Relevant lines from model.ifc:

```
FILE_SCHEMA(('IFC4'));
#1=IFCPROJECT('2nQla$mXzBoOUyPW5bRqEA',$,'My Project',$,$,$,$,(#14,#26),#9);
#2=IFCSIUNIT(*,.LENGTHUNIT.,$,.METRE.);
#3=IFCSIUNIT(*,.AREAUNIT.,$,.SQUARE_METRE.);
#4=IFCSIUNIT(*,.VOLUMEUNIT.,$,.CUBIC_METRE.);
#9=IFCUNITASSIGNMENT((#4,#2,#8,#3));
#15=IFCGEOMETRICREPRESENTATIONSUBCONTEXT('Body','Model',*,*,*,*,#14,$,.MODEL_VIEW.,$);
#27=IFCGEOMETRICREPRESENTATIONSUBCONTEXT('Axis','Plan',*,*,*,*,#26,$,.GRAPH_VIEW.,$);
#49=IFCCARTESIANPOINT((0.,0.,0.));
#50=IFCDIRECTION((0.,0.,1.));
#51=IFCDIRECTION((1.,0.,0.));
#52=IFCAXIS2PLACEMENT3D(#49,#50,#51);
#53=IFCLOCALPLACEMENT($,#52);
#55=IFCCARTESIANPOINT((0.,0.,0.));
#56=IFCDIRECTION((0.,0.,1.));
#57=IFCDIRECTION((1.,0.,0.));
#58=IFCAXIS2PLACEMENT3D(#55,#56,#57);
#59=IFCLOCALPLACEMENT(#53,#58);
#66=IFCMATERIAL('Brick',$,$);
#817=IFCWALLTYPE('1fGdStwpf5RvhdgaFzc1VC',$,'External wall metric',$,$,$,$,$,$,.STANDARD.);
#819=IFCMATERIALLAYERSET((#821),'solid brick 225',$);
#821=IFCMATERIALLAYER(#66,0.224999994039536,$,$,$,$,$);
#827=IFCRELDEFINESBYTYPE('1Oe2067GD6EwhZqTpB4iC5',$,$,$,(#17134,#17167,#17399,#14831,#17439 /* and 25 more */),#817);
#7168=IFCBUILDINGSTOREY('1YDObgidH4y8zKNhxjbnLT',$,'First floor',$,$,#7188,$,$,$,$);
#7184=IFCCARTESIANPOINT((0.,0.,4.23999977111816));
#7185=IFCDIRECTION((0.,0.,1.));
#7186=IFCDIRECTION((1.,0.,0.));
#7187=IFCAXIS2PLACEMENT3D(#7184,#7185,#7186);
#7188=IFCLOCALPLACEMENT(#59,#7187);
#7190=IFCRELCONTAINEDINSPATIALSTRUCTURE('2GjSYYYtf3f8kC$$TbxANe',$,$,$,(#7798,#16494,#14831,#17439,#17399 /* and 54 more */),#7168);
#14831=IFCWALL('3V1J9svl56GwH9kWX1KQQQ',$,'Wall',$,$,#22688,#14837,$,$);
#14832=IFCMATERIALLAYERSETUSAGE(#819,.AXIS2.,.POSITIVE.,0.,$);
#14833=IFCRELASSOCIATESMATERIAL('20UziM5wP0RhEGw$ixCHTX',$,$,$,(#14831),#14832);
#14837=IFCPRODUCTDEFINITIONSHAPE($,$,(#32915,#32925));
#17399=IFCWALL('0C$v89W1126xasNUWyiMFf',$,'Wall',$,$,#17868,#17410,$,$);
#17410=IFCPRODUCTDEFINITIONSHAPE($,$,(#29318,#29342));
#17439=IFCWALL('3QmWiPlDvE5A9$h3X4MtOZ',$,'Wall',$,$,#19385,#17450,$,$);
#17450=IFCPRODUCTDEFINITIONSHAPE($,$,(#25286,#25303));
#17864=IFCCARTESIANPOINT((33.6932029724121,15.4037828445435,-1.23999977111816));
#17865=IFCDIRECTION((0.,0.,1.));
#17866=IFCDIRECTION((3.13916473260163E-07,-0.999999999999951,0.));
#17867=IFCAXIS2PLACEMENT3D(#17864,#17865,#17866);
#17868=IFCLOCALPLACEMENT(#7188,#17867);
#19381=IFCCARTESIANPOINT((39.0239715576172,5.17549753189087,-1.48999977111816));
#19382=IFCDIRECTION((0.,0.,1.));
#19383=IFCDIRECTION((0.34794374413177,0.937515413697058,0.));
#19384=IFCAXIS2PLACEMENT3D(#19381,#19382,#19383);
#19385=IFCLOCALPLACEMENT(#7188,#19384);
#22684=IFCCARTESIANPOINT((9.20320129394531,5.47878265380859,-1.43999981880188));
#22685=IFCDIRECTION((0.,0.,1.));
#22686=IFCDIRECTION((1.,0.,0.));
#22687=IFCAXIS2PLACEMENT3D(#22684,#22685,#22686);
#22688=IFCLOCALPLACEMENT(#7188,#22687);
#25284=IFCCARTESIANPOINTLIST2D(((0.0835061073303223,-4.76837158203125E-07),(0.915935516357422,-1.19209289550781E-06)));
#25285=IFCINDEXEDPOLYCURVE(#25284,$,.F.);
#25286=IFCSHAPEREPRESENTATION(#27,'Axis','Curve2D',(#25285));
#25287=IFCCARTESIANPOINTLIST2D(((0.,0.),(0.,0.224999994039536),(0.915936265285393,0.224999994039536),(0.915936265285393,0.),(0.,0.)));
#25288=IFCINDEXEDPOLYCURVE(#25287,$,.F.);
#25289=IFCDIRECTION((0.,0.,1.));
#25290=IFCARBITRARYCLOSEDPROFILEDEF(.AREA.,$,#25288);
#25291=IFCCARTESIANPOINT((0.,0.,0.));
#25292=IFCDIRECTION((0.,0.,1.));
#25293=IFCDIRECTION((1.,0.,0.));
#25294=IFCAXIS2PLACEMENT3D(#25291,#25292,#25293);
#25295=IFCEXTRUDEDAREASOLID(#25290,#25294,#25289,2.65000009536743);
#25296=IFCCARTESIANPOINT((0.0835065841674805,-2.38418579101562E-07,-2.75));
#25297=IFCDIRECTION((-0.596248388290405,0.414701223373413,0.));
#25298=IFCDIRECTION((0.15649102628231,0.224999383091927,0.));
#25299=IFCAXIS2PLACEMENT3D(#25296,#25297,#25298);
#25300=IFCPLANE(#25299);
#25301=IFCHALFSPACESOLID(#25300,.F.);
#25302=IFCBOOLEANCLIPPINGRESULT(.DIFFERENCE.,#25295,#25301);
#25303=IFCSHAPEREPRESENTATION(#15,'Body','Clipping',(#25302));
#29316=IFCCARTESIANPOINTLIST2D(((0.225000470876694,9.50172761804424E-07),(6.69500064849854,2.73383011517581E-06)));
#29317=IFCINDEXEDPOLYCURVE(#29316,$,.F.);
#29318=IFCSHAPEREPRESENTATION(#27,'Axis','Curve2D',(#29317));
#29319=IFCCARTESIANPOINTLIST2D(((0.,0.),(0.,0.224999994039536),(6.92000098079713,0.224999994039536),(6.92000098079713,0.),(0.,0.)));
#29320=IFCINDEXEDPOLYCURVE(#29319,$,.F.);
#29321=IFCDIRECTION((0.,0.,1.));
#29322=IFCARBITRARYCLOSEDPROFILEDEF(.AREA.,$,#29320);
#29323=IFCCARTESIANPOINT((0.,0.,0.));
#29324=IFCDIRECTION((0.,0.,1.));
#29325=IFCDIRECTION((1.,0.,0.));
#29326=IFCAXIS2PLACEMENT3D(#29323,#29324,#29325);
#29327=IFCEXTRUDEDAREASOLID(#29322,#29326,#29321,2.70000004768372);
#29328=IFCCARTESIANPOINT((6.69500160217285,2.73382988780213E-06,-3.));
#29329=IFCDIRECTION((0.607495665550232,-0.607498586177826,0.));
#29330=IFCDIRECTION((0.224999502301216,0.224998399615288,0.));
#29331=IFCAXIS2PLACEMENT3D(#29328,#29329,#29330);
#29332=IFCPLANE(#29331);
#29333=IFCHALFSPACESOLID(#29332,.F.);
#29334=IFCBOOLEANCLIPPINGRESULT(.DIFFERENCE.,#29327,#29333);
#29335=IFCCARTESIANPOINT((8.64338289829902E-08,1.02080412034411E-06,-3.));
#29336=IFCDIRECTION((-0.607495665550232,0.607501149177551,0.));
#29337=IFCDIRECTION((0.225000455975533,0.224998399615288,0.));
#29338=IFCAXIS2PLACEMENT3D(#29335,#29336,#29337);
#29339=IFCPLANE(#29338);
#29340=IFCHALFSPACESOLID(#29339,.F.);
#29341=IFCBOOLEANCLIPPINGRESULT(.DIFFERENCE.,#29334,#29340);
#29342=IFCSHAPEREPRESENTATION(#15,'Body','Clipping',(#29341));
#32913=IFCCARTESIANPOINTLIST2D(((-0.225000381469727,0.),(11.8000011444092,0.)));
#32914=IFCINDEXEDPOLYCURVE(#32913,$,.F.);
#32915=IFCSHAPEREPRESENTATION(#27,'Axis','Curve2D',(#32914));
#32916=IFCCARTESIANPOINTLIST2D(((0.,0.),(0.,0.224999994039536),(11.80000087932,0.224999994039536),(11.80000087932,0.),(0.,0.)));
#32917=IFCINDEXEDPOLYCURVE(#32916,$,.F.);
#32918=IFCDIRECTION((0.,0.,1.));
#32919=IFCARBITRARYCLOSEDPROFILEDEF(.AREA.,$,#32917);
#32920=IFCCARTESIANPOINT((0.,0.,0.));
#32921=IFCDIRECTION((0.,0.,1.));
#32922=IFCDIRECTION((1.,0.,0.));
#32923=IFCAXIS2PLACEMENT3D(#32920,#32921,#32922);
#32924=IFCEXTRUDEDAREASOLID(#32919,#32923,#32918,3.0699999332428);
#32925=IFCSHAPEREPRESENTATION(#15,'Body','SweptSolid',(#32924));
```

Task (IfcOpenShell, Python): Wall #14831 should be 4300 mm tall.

```python
import ifcopenshell
import ifcopenshell.geom
import ifcopenshell.util.representation
import ifcopenshell.util.shape
import ifcopenshell.util.unit

model = ifcopenshell.open("model.ifc")
unit_scale = ifcopenshell.util.unit.calculate_unit_scale(model)
settings = ifcopenshell.geom.settings()


def volume(element):
    """Net volume in cubic metres, openings subtracted."""
    shape = ifcopenshell.geom.create_shape(settings, element)
    return ifcopenshell.util.shape.get_volume(shape.geometry)


wall = model.by_guid("3V1J9svl56GwH9kWX1KQQQ")
before = volume(wall)

body = ifcopenshell.util.representation.get_representation(wall, "Model", "Body")
solid = body.Items[0]
old_height = solid.Depth
solid.Depth = 4.3 / unit_scale
after = volume(wall)

print(f"height {old_height:g} -> {solid.Depth:g}, volume {before:.3f} -> {after:.3f} m3")

model.write("model_v2.ifc")
```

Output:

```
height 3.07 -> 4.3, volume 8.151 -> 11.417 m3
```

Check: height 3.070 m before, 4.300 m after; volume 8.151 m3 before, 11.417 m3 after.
